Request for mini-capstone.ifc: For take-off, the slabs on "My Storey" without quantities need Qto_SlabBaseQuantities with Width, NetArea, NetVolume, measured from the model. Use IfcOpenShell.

First a look at what the model holds.

```python
import ifcopenshell
import ifcopenshell.util.element
import ifcopenshell.util.unit

model = ifcopenshell.open("mini-capstone.ifc")
print(model.schema)
for unit_type in ("LENGTHUNIT", "AREAUNIT", "VOLUMEUNIT"):
    print(unit_type, ifcopenshell.util.unit.calculate_unit_scale(model, unit_type))
storey = next(s for s in model.by_type("IfcBuildingStorey") if s.Name == "My Storey")
slabs = [e for e in ifcopenshell.util.element.get_decomposition(storey) if e.is_a("IfcSlab")]
for e in sorted(slabs, key=lambda e: e.id()):
    print(e.id(), e.is_a(), e.Name, list(ifcopenshell.util.element.get_psets(e, qtos_only=True)), sep=" | ")
```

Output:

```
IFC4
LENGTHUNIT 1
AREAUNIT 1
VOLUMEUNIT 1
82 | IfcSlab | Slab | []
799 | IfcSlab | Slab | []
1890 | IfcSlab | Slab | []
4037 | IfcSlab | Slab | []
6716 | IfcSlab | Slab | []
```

```python
import ifcopenshell
import ifcopenshell.api.pset
import ifcopenshell.geom
import ifcopenshell.util.element
import ifcopenshell.util.shape
import ifcopenshell.util.unit

model = ifcopenshell.open("mini-capstone.ifc")
unit_scale = ifcopenshell.util.unit.calculate_unit_scale(model)
area_scale = ifcopenshell.util.unit.calculate_unit_scale(model, "AREAUNIT")
volume_scale = ifcopenshell.util.unit.calculate_unit_scale(model, "VOLUMEUNIT")
settings = ifcopenshell.geom.settings()

storey = next(s for s in model.by_type("IfcBuildingStorey") if s.Name == "My Storey")
slabs = [e for e in ifcopenshell.util.element.get_decomposition(storey) if e.is_a("IfcSlab")]

for e in sorted(slabs, key=lambda e: e.id()):
    if ifcopenshell.util.element.get_psets(e, qtos_only=True, should_inherit=False):
        continue
    # Geometry comes back in metres, in the element's own axes.
    shape = ifcopenshell.geom.create_shape(settings, e)
    values = {
        "Width": ifcopenshell.util.shape.get_z(shape.geometry) / unit_scale,
        "NetArea": ifcopenshell.util.shape.get_footprint_area(shape.geometry) / area_scale,
        "NetVolume": ifcopenshell.util.shape.get_volume(shape.geometry) / volume_scale,
    }
    qto = ifcopenshell.api.pset.add_qto(model, product=e, name="Qto_SlabBaseQuantities")
    ifcopenshell.api.pset.edit_qto(model, qto=qto, properties=values)
    print(e.id(), {k: round(v, 3) for k, v in values.items()})

model.write("mini-capstone_edited.ifc")
```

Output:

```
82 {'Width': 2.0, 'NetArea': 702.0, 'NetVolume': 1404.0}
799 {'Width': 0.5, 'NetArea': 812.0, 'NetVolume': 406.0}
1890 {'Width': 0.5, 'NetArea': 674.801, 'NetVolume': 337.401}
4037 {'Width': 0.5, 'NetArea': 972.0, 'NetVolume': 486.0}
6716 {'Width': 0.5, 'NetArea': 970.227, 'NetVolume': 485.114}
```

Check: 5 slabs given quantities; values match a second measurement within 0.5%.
